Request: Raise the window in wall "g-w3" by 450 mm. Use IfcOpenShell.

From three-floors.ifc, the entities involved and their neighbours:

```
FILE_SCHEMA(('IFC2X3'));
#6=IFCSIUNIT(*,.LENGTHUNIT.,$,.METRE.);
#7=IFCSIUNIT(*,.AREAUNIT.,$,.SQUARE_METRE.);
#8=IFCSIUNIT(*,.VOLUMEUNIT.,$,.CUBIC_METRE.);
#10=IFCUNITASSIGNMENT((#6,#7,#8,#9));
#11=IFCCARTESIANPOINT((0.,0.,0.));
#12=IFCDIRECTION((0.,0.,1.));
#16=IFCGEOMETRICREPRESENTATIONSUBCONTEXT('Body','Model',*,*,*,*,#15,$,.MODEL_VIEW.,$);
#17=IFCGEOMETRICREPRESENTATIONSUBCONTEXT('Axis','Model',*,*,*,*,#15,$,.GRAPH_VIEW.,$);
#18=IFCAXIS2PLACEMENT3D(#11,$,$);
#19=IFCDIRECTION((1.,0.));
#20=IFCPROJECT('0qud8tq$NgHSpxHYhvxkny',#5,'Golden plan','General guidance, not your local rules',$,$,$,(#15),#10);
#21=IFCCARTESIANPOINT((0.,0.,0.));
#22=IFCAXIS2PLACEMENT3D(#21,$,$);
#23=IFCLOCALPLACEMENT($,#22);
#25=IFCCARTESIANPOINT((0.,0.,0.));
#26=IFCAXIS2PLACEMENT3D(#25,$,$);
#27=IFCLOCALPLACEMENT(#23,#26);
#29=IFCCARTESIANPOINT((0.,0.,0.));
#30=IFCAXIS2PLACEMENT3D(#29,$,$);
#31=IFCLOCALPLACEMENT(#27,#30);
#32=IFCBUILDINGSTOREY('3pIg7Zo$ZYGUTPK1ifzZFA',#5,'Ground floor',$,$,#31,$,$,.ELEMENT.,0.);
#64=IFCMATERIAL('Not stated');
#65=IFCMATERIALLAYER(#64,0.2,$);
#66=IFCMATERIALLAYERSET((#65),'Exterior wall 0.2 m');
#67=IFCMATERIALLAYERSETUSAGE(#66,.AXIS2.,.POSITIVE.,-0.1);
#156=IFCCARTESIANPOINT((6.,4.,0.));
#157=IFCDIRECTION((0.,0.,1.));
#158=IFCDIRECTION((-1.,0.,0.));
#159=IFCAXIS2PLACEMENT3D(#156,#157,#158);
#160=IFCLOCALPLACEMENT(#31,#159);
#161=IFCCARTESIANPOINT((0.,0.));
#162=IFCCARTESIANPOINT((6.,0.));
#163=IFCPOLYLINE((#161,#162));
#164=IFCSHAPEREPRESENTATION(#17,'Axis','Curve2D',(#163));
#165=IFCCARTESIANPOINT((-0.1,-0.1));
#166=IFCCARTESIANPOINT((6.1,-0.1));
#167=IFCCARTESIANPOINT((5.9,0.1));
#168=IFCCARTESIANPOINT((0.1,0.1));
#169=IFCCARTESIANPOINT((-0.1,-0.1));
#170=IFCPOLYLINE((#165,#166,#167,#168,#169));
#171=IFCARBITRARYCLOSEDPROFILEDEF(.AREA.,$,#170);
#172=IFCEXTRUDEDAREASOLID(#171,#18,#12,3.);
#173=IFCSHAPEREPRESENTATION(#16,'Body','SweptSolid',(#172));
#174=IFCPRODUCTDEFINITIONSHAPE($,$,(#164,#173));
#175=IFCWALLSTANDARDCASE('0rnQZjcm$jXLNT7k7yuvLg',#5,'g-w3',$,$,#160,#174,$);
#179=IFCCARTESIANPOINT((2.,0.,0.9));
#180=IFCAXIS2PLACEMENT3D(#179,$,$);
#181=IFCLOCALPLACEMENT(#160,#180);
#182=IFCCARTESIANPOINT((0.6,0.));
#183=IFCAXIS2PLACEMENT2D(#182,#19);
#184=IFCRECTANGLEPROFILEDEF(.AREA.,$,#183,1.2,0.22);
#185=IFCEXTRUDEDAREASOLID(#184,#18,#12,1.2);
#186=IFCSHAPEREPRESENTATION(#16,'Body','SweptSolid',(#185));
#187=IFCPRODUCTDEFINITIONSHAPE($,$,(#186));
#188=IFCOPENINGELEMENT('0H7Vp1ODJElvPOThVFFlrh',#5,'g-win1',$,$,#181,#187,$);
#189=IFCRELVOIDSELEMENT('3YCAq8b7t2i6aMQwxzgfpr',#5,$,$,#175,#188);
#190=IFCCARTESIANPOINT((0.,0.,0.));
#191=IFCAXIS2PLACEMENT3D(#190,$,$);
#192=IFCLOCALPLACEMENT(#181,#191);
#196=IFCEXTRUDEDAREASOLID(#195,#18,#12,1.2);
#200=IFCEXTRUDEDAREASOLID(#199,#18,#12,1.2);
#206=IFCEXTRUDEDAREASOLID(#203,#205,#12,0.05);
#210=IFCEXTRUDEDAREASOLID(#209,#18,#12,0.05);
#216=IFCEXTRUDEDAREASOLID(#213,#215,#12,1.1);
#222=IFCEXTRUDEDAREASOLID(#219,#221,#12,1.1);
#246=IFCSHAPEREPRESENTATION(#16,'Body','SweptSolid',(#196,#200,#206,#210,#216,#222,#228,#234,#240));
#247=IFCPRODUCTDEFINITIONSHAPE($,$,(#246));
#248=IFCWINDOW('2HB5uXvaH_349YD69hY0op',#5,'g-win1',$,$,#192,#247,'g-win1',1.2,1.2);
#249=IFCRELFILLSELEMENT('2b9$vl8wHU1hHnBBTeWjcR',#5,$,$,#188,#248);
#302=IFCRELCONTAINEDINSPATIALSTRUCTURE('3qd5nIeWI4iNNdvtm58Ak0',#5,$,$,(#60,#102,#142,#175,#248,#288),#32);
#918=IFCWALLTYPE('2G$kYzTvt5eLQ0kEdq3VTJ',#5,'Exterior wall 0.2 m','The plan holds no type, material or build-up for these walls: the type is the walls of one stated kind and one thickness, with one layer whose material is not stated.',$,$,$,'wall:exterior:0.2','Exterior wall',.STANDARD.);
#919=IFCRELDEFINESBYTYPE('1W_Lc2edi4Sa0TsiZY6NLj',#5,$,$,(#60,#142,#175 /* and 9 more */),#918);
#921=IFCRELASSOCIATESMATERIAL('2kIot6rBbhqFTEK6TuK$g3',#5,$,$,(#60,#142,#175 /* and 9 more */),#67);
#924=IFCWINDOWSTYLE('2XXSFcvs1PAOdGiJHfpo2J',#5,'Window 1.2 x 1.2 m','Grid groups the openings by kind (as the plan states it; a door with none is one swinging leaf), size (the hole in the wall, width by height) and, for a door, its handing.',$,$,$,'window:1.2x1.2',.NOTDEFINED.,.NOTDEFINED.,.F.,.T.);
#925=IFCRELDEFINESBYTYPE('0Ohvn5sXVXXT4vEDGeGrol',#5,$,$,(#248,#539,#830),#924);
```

```python
import numpy as np
import ifcopenshell
import ifcopenshell.api.geometry
import ifcopenshell.util.placement
import ifcopenshell.util.unit

model = ifcopenshell.open("three-floors.ifc")
unit_scale = ifcopenshell.util.unit.calculate_unit_scale(model)

window = model.by_guid("2HB5uXvaH_349YD69hY0op")
opening = window.FillsVoids[0].RelatingOpeningElement
dz = 0.45

shift = np.array([0.0, 0.0, dz])
# The window is placed relative to its opening, so it follows when the opening moves.
matrix = ifcopenshell.util.placement.get_local_placement(opening.ObjectPlacement)
matrix[:3, 3] += shift
ifcopenshell.api.geometry.edit_object_placement(
    model, product=opening, matrix=matrix, is_si=False, should_transform_children=True
)

print(f"moved by {dz * unit_scale:+.3f} m")

model.write("three-floors-out.ifc")
```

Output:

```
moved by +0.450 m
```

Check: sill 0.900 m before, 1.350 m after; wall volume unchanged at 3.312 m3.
